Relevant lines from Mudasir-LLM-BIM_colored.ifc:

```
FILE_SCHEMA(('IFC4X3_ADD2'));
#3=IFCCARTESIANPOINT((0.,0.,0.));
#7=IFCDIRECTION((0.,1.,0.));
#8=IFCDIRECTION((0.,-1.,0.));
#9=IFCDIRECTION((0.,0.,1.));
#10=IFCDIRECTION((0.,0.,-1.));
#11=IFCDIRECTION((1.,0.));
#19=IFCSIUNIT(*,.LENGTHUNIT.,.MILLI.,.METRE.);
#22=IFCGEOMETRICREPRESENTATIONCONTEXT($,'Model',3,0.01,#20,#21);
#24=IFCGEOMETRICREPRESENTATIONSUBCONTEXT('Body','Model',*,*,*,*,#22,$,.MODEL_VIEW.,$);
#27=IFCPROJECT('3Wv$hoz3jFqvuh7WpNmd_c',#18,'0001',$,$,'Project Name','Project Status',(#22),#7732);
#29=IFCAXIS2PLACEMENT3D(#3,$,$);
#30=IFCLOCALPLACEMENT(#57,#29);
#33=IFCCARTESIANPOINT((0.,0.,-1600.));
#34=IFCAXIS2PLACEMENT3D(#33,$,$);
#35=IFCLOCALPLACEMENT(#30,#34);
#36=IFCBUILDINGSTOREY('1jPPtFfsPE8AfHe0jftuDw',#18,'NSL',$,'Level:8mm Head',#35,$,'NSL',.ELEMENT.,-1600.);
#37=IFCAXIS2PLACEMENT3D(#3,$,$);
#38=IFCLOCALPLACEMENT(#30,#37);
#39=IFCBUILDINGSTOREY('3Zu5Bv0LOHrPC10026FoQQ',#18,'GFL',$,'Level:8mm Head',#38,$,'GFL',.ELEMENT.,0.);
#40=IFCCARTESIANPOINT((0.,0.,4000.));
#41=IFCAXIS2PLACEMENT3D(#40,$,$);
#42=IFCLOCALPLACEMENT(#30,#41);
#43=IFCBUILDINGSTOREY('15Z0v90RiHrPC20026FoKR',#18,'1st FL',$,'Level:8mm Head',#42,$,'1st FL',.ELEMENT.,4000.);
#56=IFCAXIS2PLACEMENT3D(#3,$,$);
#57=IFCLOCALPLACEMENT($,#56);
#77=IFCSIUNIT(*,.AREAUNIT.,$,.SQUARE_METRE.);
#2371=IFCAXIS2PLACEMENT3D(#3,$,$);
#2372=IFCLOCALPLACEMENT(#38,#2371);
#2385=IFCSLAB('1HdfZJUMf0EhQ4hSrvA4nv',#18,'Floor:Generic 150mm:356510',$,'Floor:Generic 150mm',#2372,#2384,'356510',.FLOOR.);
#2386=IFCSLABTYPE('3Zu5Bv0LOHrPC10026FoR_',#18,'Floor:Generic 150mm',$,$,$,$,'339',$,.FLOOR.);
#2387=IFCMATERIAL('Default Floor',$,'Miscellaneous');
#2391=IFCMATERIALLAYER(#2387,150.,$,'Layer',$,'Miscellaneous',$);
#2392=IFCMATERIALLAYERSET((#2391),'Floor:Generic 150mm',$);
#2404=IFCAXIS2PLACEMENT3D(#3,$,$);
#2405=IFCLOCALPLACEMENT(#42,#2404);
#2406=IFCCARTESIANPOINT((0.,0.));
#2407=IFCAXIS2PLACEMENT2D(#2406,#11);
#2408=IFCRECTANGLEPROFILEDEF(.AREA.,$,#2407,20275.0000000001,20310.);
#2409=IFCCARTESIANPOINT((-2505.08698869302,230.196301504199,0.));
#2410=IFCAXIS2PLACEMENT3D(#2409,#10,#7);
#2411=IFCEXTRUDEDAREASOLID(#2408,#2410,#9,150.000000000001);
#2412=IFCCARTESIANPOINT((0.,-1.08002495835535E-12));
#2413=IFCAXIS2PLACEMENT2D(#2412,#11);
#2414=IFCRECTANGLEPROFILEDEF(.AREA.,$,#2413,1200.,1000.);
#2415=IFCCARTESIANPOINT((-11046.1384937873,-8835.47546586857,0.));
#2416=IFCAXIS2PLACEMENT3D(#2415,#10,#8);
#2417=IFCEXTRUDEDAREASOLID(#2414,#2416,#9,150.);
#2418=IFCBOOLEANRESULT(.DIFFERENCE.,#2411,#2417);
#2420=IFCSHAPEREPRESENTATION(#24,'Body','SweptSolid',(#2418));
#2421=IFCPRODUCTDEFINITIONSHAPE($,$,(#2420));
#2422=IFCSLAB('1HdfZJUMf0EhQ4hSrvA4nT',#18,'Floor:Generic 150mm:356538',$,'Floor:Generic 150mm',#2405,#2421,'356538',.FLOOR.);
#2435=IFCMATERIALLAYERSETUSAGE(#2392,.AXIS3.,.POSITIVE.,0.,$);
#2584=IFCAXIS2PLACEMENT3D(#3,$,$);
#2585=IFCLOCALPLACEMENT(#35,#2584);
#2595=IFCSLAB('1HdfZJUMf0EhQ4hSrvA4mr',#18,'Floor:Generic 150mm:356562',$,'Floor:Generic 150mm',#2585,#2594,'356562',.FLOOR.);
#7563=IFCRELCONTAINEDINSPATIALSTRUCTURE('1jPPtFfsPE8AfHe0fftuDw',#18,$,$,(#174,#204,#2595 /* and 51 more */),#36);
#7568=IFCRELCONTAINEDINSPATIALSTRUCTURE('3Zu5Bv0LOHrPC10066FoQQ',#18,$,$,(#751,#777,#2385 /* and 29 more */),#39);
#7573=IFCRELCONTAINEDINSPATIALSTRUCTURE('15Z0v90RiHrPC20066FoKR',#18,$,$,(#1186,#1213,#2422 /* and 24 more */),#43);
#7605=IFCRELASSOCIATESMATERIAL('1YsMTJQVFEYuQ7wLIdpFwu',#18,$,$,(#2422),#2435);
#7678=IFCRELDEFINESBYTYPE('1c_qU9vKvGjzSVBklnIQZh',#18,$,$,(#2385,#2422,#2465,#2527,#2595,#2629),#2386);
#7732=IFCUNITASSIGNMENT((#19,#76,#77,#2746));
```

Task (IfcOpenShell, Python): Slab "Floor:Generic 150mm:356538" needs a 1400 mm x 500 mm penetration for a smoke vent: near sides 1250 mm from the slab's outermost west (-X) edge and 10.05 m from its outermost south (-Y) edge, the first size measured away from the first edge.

```python
import numpy as np
import ifcopenshell
import ifcopenshell.api.feature
import ifcopenshell.api.geometry
import ifcopenshell.api.root
import ifcopenshell.geom
import ifcopenshell.util.placement
import ifcopenshell.util.representation
import ifcopenshell.util.shape
import ifcopenshell.util.unit

model = ifcopenshell.open("Mudasir-LLM-BIM_colored.ifc")
unit_scale = ifcopenshell.util.unit.calculate_unit_scale(model)
settings = ifcopenshell.geom.settings()


def volume(element):
    """Net volume in cubic metres, openings subtracted."""
    shape = ifcopenshell.geom.create_shape(settings, element)
    return ifcopenshell.util.shape.get_volume(shape.geometry)


slab = model.by_guid("1HdfZJUMf0EhQ4hSrvA4nT")
before = volume(slab)

# Extent in the slab's own axes, in metres. The edges named are its -X and -Y sides.
slab_shape = ifcopenshell.geom.create_shape(settings, slab)
vertices = ifcopenshell.util.shape.get_vertices(slab_shape.geometry)
x_min, y_min, bottom = vertices.min(axis=0)
top = vertices[:, 2].max()

opening = ifcopenshell.api.root.create_entity(model, ifc_class="IfcOpeningElement", name="Smoke vent opening", predefined_type="OPENING")
context = ifcopenshell.util.representation.get_context(model, "Model", "Body", "MODEL_VIEW")
width, depth = 1.4, 0.5
outline = [(0.0, 0.0), (width, 0.0), (width, depth), (0.0, depth), (0.0, 0.0)]
# Overshoot both faces by 50 mm so the cut is clean.
shape = ifcopenshell.api.geometry.add_slab_representation(
    model, context=context, depth=top - bottom + 0.1, polyline=outline
)
ifcopenshell.api.geometry.assign_representation(model, product=opening, representation=shape)

matrix = ifcopenshell.util.placement.get_local_placement(slab.ObjectPlacement)
matrix[:, 3] = matrix @ np.append(np.array([x_min + 1.25, y_min + 10.05, bottom - 0.05]) / unit_scale, 1.0)
ifcopenshell.api.geometry.edit_object_placement(model, product=opening, matrix=matrix, is_si=False)
ifcopenshell.api.feature.add_feature(model, feature=opening, element=slab)

after = volume(slab)

print(f"slab volume {before:.3f} -> {after:.3f} m3")

model.write("Mudasir-LLM-BIM_colored_rev.ifc")
```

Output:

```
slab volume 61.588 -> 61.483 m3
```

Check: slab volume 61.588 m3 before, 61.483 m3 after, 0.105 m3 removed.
